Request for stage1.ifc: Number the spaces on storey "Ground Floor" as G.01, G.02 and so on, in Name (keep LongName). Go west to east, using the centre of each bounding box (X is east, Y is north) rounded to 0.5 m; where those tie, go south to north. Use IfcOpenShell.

First a look at what the model holds.

```python
import ifcopenshell
import ifcopenshell.util.element
import ifcopenshell.util.placement

model = ifcopenshell.open("stage1.ifc")
print(model.schema)
storey = next(s for s in model.by_type("IfcBuildingStorey") if s.Name == "Ground Floor")
spaces = [e for e in ifcopenshell.util.element.get_decomposition(storey) if e.is_a("IfcSpace")]
for e in sorted(spaces, key=lambda e: e.id()):
    origin = ifcopenshell.util.placement.get_local_placement(e.ObjectPlacement)[:3, 3]
    print(e.id(), e.Name, e.LongName, origin.round(2) + 0.0, sep=" | ")
```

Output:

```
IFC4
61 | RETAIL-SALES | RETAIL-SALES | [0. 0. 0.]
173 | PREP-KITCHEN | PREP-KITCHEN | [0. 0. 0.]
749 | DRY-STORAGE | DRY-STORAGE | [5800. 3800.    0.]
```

```python
import ifcopenshell
import ifcopenshell.geom
import ifcopenshell.util.element
import ifcopenshell.util.shape

model = ifcopenshell.open("stage1.ifc")
settings = ifcopenshell.geom.settings()
settings.set("use-world-coords", True)


def centre(element):
    shape = ifcopenshell.geom.create_shape(settings, element)
    return ifcopenshell.util.shape.get_bbox_centroid(shape.geometry)


storey = next(s for s in model.by_type("IfcBuildingStorey") if s.Name == "Ground Floor")
spaces = [e for e in ifcopenshell.util.element.get_decomposition(storey) if e.is_a("IfcSpace")]

# Insertion points can sit at a corner or the storey origin, so sort by the geometry (in metres).
centres = {e: centre(e) for e in spaces}
spaces.sort(key=lambda e: (round(centres[e][0] / 0.5), centres[e][1]))

for i, e in enumerate(spaces, start=1):
    number = f"G.{i:02d}"
    e.Name = number
    print(e.id(), number)

model.write("stage1_rev.ifc")
```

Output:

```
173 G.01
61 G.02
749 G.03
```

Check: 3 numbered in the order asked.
